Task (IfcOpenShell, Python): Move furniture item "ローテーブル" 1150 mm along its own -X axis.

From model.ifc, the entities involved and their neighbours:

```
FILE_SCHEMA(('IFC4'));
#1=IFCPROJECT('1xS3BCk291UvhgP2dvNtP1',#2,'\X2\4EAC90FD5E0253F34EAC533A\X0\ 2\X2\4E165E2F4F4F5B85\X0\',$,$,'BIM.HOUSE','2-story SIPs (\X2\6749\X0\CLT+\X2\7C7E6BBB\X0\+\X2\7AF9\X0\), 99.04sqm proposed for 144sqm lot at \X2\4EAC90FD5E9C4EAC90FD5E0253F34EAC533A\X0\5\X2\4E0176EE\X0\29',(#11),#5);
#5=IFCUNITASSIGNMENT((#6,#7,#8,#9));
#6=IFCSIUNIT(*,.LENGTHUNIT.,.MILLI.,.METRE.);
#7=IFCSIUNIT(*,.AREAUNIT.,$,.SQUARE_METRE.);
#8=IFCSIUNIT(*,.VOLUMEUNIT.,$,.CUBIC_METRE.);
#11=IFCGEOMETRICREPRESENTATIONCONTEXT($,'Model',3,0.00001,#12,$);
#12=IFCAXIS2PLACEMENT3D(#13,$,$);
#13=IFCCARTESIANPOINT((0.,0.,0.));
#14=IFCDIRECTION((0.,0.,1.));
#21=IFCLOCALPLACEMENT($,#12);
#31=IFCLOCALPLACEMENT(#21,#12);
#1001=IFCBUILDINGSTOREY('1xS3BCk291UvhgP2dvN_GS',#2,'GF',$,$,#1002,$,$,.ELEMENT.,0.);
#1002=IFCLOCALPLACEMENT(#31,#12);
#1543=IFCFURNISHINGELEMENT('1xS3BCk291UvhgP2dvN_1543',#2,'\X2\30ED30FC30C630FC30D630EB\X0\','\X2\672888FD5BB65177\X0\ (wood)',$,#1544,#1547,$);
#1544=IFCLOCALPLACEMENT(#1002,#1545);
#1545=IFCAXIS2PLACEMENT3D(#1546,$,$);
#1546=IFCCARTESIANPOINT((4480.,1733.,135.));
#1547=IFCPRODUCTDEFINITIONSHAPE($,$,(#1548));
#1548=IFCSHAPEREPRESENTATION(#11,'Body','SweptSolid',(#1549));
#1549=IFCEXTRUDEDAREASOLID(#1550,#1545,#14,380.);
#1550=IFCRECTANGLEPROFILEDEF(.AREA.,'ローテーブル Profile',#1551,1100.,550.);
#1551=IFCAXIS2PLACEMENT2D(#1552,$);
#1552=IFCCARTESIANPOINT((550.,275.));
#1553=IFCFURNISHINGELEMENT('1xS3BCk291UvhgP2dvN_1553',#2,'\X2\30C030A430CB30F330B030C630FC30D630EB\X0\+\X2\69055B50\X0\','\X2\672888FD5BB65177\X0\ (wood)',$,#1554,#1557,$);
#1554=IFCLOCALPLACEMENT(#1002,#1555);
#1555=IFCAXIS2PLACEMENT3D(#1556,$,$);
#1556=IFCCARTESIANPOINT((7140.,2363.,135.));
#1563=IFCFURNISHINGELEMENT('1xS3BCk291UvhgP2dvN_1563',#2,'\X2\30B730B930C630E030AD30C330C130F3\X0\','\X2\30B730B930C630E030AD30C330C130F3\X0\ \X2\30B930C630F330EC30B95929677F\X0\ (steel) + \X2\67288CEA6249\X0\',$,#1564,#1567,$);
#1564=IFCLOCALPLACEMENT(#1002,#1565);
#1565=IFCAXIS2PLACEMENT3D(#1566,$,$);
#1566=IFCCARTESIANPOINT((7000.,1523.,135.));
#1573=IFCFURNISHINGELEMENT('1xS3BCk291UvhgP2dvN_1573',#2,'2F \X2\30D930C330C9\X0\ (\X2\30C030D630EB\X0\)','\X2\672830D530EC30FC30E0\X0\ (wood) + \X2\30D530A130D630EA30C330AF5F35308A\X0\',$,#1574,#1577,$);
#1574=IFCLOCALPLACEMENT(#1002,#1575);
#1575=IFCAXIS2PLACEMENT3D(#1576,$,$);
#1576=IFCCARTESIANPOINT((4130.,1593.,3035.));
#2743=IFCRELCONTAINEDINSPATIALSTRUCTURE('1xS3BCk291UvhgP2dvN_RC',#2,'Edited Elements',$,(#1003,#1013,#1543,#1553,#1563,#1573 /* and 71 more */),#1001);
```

```python
import ifcopenshell
import ifcopenshell.api.geometry
import ifcopenshell.util.placement
import ifcopenshell.util.unit

model = ifcopenshell.open("model.ifc")
unit_scale = ifcopenshell.util.unit.calculate_unit_scale(model)

item = model.by_guid("1xS3BCk291UvhgP2dvN_1543")
matrix = ifcopenshell.util.placement.get_local_placement(item.ObjectPlacement)
matrix[:3, 3] -= matrix[:3, 0] * 1.15 / unit_scale
ifcopenshell.api.geometry.edit_object_placement(model, product=item, matrix=matrix, is_si=False)

print(ifcopenshell.util.placement.get_local_placement(item.ObjectPlacement).round(3) + 0.0)

model.write("model_edited.ifc")
```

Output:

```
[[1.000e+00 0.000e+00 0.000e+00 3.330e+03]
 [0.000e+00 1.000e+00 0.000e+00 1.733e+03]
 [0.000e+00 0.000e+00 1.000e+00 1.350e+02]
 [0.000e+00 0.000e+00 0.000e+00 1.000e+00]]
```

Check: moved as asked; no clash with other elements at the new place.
